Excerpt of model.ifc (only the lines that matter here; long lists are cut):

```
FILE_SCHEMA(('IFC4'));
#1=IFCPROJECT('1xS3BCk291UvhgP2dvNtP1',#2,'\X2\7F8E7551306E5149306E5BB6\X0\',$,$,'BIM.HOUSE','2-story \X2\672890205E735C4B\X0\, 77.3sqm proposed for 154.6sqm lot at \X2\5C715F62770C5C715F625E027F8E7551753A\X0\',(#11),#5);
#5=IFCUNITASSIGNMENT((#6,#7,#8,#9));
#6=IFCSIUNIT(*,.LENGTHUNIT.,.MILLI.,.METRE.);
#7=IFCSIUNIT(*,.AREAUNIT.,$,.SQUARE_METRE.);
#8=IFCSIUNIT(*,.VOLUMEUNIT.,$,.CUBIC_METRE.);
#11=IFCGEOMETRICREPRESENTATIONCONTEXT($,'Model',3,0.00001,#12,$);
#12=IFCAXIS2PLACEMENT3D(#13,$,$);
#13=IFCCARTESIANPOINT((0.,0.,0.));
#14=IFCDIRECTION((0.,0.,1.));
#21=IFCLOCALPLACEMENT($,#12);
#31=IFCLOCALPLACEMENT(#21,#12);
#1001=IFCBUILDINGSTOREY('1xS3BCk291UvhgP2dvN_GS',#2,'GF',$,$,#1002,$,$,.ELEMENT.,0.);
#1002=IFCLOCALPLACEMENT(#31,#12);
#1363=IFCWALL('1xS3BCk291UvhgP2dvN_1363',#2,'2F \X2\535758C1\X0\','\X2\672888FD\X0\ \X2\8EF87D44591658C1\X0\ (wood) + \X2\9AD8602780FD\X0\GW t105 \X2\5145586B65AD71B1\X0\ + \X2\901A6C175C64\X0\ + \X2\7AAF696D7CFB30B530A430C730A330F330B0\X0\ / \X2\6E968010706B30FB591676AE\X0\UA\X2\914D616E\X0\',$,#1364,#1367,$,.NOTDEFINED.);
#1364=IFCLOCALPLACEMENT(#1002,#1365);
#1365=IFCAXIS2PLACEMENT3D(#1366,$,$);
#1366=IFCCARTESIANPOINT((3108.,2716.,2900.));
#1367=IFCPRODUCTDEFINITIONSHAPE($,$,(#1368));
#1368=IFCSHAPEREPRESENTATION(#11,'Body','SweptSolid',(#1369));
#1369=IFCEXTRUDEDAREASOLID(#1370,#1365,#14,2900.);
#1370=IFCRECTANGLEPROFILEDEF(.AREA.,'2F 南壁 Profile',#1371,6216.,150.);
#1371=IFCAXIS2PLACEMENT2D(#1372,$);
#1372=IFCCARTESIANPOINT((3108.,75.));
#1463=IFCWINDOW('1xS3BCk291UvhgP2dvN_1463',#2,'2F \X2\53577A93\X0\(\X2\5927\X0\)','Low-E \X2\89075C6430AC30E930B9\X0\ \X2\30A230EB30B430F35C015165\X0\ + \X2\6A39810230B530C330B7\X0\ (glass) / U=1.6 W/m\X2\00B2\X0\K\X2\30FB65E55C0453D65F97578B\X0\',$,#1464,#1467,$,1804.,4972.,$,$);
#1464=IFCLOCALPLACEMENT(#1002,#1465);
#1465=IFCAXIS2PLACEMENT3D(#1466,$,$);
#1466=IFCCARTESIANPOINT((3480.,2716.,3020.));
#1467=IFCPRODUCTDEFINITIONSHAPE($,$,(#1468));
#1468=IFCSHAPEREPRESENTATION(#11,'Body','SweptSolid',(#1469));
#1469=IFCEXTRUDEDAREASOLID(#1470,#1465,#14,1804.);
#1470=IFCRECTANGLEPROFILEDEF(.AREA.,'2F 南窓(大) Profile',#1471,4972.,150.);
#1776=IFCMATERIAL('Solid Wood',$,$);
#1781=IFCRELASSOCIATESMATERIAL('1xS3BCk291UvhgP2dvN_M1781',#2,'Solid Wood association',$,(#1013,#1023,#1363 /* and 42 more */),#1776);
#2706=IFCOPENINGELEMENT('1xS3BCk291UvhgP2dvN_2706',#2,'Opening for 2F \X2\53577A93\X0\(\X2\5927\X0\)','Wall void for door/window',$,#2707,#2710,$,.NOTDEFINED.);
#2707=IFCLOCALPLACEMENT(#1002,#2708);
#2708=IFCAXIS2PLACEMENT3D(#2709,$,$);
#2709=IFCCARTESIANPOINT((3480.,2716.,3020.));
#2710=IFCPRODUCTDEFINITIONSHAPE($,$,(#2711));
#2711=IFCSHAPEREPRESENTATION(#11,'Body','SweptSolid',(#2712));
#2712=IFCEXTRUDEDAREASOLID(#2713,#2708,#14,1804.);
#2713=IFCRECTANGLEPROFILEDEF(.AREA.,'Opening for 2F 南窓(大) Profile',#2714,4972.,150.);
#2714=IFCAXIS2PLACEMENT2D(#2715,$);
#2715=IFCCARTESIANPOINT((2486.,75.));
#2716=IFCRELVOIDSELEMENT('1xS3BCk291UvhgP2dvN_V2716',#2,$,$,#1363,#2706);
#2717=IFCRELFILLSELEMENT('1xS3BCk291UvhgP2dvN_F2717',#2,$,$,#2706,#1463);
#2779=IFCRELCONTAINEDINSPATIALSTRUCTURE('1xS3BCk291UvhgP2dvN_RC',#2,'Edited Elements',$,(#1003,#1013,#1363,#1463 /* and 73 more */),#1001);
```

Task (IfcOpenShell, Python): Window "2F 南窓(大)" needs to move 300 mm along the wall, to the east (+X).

```python
import ifcopenshell
import ifcopenshell.api.geometry
import ifcopenshell.util.placement
import ifcopenshell.util.unit

model = ifcopenshell.open("model.ifc")
unit_scale = ifcopenshell.util.unit.calculate_unit_scale(model)

window = model.by_guid("1xS3BCk291UvhgP2dvN_1463")
opening = window.FillsVoids[0].RelatingOpeningElement
wall = opening.VoidsElements[0].RelatingBuildingElement

wall_matrix = ifcopenshell.util.placement.get_local_placement(wall.ObjectPlacement)
shift = wall_matrix[:3, 0] * 0.3 / unit_scale
before = ifcopenshell.util.placement.get_local_placement(window.ObjectPlacement)[:3, 3].copy()

# The window is not placed relative to its opening, so move both.
for product in (opening, window):
    matrix = ifcopenshell.util.placement.get_local_placement(product.ObjectPlacement)
    matrix[:3, 3] += shift
    ifcopenshell.api.geometry.edit_object_placement(model, product=product, matrix=matrix, is_si=False)

after = ifcopenshell.util.placement.get_local_placement(window.ObjectPlacement)[:3, 3]
print("window moved by", (after - before).round(3) + 0.0)

model.write("model-out.ifc")
```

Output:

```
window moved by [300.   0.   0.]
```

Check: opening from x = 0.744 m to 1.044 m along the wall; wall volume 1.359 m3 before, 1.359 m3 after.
